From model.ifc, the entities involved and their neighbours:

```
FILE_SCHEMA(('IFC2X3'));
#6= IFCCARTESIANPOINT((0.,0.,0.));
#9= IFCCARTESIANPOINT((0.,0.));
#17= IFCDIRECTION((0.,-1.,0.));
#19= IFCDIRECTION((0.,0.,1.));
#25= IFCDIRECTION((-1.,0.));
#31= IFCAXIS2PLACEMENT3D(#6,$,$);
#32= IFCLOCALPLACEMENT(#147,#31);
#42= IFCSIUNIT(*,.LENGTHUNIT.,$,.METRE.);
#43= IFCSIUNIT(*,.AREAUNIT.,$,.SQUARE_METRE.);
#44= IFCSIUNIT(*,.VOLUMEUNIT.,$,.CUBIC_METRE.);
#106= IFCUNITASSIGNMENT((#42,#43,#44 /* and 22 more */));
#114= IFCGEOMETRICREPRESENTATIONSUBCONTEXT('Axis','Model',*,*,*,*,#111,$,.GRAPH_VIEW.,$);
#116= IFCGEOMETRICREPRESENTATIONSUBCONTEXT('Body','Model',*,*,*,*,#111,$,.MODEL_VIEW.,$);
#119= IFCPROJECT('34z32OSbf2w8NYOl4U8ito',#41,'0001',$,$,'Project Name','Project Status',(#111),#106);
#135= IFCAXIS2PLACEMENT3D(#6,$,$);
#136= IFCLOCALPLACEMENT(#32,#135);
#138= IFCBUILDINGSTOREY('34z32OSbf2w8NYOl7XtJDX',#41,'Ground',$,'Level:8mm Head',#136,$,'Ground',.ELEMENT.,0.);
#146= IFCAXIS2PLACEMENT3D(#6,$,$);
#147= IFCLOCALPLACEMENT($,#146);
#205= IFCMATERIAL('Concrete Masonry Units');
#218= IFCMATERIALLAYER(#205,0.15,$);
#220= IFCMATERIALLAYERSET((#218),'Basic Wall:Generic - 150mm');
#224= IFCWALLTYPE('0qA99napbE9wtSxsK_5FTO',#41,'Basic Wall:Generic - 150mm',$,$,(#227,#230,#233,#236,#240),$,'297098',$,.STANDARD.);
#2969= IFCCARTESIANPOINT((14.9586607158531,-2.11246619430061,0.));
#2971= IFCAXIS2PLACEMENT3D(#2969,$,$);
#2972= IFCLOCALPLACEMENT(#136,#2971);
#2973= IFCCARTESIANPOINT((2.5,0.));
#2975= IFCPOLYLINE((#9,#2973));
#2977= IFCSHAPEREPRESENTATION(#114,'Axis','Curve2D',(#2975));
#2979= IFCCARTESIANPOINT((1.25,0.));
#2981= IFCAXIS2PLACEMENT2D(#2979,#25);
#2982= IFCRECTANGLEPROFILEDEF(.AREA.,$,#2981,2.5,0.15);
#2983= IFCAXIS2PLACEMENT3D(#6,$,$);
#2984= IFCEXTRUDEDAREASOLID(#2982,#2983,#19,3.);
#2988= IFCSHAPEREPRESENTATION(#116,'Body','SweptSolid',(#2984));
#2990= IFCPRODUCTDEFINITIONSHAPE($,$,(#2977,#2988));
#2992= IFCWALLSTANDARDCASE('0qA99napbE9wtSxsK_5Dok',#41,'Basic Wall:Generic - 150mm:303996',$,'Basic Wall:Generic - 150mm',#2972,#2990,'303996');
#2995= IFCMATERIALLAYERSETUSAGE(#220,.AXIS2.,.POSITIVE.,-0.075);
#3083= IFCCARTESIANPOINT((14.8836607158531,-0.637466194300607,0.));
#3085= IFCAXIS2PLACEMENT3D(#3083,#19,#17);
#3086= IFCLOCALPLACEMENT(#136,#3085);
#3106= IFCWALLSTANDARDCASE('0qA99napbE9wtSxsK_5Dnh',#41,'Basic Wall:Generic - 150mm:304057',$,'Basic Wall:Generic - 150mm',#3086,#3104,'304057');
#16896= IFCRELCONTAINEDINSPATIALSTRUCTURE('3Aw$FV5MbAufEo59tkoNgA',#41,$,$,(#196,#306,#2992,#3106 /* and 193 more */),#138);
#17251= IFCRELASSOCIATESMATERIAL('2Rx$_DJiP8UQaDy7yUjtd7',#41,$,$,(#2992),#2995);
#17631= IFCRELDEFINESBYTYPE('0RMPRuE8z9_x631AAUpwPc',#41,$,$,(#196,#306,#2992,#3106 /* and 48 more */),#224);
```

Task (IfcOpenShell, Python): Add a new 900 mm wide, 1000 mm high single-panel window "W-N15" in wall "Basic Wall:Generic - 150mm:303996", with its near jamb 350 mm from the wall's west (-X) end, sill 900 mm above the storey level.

```python
import numpy as np
import ifcopenshell
import ifcopenshell.api.feature
import ifcopenshell.api.geometry
import ifcopenshell.api.root
import ifcopenshell.api.spatial
import ifcopenshell.api.type
import ifcopenshell.geom
import ifcopenshell.util.element
import ifcopenshell.util.placement
import ifcopenshell.util.representation
import ifcopenshell.util.shape
import ifcopenshell.util.unit

model = ifcopenshell.open("model.ifc")
unit_scale = ifcopenshell.util.unit.calculate_unit_scale(model)
settings = ifcopenshell.geom.settings()


def volume(element):
    """Net volume in cubic metres, openings subtracted."""
    shape = ifcopenshell.geom.create_shape(settings, element)
    return ifcopenshell.util.shape.get_volume(shape.geometry)


wall = model.by_guid("0qA99napbE9wtSxsK_5Dok")
storey = ifcopenshell.util.element.get_container(wall, ifc_class="IfcBuildingStorey")
context = ifcopenshell.util.representation.get_context(model, "Model", "Body", "MODEL_VIEW")
before = volume(wall)

width, height, from_end, sill = 0.9, 1, 0.35, 0.9  # metres

# The wall runs along its own X axis, and the end named is its -X end.
wall_shape = ifcopenshell.geom.create_shape(settings, wall)
x, y, z = ifcopenshell.util.shape.get_vertices(wall_shape.geometry).T
start = x.min() + from_end
face, thickness = float(y.min()), float(y.max() - y.min())
wall_matrix = ifcopenshell.util.placement.get_local_placement(wall.ObjectPlacement)
level = ifcopenshell.util.placement.get_local_placement(storey.ObjectPlacement)[2, 3]


def in_wall(x, y):
    """Placement at x, y metres in the wall's axes, at sill height."""
    matrix = wall_matrix.copy()
    matrix[:, 3] = wall_matrix @ np.array([x / unit_scale, y / unit_scale, 0.0, 1.0])
    matrix[2, 3] = level + sill / unit_scale
    return matrix


# Opening: a box that overshoots both wall faces by 50 mm.
opening = ifcopenshell.api.root.create_entity(model, ifc_class="IfcOpeningElement")
box = ifcopenshell.api.geometry.add_wall_representation(
    model, context=context, length=width, height=height, thickness=thickness + 0.1
)
ifcopenshell.api.geometry.assign_representation(model, product=opening, representation=box)
ifcopenshell.api.geometry.edit_object_placement(model, product=opening, matrix=in_wall(start, face - 0.05), is_si=False)
ifcopenshell.api.feature.add_feature(model, feature=opening, element=wall)

window = ifcopenshell.api.root.create_entity(model, ifc_class="IfcWindow", name="W-N15")
window.OverallWidth, window.OverallHeight = width / unit_scale, height / unit_scale
body = ifcopenshell.api.geometry.add_window_representation(
    model,
    context=context,
    overall_width=window.OverallWidth,
    overall_height=window.OverallHeight,
    partition_type="SINGLE_PANEL",
)
ifcopenshell.api.geometry.assign_representation(model, product=window, representation=body)
ifcopenshell.api.spatial.assign_container(model, products=[window], relating_structure=storey)
fills = ifcopenshell.api.feature.add_filling(model, opening=opening, element=window)
fills.OwnerHistory = window.OwnerHistory  # required in IFC2X3

# IFC2X3 keeps the operation on the window style.
style = ifcopenshell.api.root.create_entity(model, ifc_class="IfcWindowStyle", name="W-N15")
style.OperationType, style.ConstructionType = "SINGLE_PANEL", "NOTDEFINED"
style.ParameterTakesPrecedence = style.Sizeable = False
ifcopenshell.api.type.assign_type(model, related_objects=[window], relating_type=style)

# Centre the window in the wall's thickness.
ifcopenshell.api.geometry.edit_object_placement(model, product=window, matrix=in_wall(start, face), is_si=False)
window_shape = ifcopenshell.geom.create_shape(settings, window)
depth = ifcopenshell.util.shape.get_vertices(window_shape.geometry)[:, 1]
offset = face + thickness / 2 - (depth.min() + depth.max()) / 2
ifcopenshell.api.geometry.edit_object_placement(model, product=window, matrix=in_wall(start, offset), is_si=False)

after = volume(wall)

print(f"wall volume {before:.3f} -> {after:.3f} m3")

model.write("model-out.ifc")
```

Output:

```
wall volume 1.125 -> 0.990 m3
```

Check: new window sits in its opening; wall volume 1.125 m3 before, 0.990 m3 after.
